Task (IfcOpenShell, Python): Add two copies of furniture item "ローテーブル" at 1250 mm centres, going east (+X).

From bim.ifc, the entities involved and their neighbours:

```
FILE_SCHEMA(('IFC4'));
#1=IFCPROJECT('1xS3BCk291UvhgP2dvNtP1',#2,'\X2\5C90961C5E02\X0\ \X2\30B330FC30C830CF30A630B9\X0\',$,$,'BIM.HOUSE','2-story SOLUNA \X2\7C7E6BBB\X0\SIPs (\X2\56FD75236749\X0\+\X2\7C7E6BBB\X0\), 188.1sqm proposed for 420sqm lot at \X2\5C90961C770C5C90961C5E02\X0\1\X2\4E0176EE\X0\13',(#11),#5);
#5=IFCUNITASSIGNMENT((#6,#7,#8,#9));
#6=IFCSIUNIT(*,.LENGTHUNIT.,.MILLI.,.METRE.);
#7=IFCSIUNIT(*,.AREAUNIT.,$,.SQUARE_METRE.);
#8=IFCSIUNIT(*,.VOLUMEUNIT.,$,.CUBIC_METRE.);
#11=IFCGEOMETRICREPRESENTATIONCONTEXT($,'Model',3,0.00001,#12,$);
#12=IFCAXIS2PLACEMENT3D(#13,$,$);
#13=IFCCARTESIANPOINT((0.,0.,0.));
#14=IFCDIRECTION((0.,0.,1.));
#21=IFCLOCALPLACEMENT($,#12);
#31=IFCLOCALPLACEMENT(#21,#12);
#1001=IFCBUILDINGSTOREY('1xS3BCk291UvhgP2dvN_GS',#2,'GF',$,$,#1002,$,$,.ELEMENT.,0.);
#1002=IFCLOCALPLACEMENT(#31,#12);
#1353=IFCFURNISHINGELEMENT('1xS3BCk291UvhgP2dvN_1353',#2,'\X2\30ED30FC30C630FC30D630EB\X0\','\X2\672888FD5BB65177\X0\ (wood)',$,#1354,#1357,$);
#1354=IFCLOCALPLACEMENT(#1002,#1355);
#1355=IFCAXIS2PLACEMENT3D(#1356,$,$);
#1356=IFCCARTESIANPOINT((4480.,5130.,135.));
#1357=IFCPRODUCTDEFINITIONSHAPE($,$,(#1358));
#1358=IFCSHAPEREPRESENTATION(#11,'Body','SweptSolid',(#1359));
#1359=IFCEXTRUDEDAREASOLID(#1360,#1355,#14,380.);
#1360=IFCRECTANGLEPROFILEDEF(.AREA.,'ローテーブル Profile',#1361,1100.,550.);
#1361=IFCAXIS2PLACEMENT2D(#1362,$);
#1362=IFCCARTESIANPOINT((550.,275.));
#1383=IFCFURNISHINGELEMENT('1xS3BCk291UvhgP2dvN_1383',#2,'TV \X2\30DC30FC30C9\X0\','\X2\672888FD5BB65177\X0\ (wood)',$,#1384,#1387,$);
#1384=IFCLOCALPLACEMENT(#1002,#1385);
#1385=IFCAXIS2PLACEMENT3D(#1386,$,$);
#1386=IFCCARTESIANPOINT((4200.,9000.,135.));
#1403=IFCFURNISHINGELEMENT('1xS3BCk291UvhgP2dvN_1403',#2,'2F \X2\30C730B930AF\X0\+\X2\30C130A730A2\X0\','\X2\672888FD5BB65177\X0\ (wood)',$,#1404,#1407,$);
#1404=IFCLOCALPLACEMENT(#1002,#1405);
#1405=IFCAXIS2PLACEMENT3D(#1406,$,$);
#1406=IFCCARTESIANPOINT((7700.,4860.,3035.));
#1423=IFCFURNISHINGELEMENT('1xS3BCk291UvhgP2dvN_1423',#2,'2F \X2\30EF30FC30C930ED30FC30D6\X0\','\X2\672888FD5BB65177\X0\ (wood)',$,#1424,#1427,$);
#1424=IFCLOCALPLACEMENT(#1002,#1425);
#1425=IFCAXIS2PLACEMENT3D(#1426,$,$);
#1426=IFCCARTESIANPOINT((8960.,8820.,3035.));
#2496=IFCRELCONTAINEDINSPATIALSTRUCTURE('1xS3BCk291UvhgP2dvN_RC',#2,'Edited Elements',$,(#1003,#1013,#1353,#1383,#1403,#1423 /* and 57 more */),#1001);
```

```python
import numpy as np
import ifcopenshell
import ifcopenshell.api.geometry
import ifcopenshell.api.root
import ifcopenshell.util.element
import ifcopenshell.util.placement

model = ifcopenshell.open("bim.ifc")


def reuse_history(source, copy):
    """copy_class also copies each property set's owner history, people and application; keep the originals."""
    for rel in copy.IsDefinedBy:
        if rel.is_a("IfcRelDefinesByProperties") and (history := rel.RelatingPropertyDefinition.OwnerHistory):
            rel.RelatingPropertyDefinition.OwnerHistory = source.OwnerHistory
            ifcopenshell.util.element.remove_deep2(model, history)


source = model.by_guid("1xS3BCk291UvhgP2dvN_1353")
base = ifcopenshell.util.placement.get_local_placement(source.ObjectPlacement)
step = np.array([1.0, 0.0, 0.0]) * 1250.0

for i in range(1, 3):
    copy = ifcopenshell.api.root.copy_class(model, product=source)
    copy.Representation = ifcopenshell.util.element.copy_deep(
        model, source.Representation, exclude=["IfcGeometricRepresentationContext", "IfcRepresentationMap"]
    )
    reuse_history(source, copy)
    matrix = base.copy()
    matrix[:3, 3] += i * step
    print("added at", matrix[:3, 3].round(3) + 0.0)
    ifcopenshell.api.geometry.edit_object_placement(model, product=copy, matrix=matrix, is_si=False)

model.write("bim-out.ifc")
```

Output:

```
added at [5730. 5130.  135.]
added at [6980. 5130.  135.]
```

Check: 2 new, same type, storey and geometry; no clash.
